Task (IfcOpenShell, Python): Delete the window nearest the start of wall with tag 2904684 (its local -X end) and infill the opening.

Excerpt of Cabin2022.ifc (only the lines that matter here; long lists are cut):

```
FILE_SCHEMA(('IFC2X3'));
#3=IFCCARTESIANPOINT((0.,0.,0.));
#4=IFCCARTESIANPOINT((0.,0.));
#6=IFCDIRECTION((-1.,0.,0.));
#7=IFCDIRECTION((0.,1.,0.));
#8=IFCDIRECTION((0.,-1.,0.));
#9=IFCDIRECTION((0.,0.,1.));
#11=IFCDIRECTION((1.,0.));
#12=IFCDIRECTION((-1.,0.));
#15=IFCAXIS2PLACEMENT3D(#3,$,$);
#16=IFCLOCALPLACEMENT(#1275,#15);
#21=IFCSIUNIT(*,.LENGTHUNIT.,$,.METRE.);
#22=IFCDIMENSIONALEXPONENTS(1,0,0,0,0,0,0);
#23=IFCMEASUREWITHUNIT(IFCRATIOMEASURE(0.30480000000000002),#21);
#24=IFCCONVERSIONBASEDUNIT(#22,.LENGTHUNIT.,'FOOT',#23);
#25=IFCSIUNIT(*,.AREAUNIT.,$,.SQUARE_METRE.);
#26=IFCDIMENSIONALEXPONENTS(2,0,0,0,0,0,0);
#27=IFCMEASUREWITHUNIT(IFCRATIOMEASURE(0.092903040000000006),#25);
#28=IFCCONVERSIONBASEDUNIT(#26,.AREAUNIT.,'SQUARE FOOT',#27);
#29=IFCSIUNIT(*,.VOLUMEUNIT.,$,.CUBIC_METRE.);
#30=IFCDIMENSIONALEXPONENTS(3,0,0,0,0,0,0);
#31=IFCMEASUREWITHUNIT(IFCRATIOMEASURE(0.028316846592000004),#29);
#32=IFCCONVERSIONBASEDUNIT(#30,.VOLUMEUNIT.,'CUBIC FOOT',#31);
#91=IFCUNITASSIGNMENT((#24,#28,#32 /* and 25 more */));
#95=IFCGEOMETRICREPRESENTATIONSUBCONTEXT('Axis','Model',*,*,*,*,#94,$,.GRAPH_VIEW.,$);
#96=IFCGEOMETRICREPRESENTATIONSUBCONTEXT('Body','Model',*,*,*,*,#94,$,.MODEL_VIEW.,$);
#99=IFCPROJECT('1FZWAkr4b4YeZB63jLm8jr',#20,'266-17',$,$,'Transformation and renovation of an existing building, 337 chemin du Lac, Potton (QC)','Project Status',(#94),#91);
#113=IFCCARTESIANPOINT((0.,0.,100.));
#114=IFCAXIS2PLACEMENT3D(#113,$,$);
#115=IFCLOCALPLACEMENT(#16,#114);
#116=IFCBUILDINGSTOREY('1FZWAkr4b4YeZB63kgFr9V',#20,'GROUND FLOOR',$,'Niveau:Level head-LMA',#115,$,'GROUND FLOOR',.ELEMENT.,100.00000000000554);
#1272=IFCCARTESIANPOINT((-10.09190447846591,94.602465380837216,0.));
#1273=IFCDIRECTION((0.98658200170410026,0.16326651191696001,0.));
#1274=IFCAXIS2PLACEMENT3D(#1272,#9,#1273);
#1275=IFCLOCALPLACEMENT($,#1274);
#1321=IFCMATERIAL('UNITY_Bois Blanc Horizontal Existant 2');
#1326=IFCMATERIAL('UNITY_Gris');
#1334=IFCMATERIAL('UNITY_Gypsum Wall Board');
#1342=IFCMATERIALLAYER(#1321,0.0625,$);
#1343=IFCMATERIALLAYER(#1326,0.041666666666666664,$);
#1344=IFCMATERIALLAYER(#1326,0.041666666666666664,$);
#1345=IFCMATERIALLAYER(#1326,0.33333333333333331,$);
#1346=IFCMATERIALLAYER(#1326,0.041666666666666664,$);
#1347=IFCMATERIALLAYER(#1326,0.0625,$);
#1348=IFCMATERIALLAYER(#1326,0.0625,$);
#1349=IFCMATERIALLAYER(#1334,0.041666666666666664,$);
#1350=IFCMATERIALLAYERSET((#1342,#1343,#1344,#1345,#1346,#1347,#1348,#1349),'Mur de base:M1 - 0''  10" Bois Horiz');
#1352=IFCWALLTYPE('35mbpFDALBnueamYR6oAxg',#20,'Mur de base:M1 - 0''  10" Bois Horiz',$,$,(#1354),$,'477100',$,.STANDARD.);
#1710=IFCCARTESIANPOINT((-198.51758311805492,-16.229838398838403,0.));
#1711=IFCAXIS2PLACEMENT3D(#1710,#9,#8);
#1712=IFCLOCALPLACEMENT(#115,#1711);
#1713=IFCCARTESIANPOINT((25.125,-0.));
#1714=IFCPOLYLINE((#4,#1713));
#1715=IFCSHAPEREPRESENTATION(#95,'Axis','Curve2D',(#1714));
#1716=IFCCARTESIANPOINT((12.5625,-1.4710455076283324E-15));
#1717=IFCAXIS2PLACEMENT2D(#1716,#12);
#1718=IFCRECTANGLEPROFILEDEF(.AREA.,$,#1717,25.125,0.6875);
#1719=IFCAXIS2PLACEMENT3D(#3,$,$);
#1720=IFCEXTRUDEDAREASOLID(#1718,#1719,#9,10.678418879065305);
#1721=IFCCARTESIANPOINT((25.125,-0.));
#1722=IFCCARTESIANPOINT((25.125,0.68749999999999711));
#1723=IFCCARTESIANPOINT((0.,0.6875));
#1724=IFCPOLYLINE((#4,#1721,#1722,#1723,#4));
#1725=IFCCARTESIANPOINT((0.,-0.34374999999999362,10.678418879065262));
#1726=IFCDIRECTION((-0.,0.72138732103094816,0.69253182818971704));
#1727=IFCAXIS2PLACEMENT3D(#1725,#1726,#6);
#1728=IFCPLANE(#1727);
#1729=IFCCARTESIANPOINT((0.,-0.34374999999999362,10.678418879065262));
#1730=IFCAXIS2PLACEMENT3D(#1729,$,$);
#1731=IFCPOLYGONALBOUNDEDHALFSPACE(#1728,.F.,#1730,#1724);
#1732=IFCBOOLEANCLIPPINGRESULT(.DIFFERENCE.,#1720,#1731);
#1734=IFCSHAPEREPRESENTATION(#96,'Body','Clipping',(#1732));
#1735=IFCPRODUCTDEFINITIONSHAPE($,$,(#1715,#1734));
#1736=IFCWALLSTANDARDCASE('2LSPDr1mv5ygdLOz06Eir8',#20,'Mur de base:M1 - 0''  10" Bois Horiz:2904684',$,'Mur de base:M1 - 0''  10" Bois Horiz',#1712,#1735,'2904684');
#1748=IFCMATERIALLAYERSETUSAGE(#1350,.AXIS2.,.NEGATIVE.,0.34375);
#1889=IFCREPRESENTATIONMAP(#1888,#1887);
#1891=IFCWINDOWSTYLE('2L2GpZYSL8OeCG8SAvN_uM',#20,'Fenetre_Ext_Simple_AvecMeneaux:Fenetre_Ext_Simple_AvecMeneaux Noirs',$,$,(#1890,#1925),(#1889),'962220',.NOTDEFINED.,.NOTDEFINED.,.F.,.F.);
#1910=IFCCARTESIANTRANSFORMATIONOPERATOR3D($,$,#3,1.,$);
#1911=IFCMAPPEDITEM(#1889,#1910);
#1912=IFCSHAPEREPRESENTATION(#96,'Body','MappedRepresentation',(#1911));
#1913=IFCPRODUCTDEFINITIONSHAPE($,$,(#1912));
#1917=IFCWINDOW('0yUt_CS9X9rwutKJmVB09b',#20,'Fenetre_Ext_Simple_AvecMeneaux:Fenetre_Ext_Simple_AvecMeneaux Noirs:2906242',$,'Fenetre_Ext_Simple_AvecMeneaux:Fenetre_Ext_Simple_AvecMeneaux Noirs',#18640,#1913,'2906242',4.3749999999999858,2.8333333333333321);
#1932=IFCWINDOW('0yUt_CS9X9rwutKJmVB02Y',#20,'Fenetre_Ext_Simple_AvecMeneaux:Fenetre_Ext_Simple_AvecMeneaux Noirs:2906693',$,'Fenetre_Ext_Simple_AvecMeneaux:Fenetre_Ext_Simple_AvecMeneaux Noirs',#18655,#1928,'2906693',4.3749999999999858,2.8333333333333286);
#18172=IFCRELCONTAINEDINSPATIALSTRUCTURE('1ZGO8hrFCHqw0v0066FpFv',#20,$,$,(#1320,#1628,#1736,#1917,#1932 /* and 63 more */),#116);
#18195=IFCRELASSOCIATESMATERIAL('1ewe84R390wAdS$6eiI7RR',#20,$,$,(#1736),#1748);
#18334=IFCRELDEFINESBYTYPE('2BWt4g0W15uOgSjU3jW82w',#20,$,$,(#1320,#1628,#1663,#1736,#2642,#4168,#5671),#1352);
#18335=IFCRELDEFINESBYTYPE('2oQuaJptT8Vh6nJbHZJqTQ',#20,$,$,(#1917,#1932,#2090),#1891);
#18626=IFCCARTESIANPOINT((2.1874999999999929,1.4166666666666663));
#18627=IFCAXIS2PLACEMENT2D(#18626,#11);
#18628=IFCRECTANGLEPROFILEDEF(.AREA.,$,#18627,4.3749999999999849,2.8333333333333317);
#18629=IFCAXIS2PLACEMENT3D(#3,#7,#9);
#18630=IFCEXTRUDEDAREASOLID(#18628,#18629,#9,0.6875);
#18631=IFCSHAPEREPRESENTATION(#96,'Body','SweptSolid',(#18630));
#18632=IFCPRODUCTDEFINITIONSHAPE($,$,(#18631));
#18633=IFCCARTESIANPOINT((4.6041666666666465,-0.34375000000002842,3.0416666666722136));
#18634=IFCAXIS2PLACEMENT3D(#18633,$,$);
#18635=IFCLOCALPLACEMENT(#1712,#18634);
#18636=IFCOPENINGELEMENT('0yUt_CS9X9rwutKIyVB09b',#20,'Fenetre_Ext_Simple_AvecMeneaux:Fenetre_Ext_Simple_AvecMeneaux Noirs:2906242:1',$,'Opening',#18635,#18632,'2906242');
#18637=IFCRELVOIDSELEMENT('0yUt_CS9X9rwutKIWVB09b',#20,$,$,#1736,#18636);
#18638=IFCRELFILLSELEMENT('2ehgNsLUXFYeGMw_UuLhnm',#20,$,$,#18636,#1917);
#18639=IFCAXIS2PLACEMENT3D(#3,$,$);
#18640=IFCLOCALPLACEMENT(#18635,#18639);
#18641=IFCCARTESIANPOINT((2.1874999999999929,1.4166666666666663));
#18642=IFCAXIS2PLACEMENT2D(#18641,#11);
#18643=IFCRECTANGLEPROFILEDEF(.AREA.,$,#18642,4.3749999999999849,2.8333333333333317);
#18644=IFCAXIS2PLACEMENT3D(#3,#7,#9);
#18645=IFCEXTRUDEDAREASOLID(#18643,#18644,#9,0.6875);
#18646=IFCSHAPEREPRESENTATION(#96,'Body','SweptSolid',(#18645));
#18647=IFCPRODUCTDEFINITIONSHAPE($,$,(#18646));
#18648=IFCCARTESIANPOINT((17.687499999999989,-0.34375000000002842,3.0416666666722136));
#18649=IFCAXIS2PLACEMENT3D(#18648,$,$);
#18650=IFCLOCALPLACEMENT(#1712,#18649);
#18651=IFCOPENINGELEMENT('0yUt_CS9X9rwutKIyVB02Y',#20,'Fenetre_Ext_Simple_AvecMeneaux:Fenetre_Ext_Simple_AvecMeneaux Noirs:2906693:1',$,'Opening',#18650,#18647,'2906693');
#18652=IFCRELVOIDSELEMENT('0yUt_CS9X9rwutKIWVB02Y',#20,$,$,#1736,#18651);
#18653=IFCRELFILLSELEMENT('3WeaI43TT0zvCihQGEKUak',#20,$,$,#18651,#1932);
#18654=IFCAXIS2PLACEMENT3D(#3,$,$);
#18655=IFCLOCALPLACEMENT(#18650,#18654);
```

```python
import ifcopenshell
import ifcopenshell.api.feature
import ifcopenshell.api.root
import ifcopenshell.geom
import ifcopenshell.util.shape

model = ifcopenshell.open("Cabin2022.ifc")
settings = ifcopenshell.geom.settings()


def volume(element):
    """Net volume in cubic metres, openings subtracted."""
    shape = ifcopenshell.geom.create_shape(settings, element)
    return ifcopenshell.util.shape.get_volume(shape.geometry)


window = model.by_guid("0yUt_CS9X9rwutKJmVB09b")
opening = window.FillsVoids[0].RelatingOpeningElement
wall = opening.VoidsElements[0].RelatingBuildingElement
before = volume(wall)

ifcopenshell.api.root.remove_product(model, product=window)
ifcopenshell.api.feature.remove_feature(model, feature=opening)

after = volume(wall)

print(f"wall volume {before:.3f} -> {after:.3f} m3")

model.write("Cabin2022_v2.ifc")
```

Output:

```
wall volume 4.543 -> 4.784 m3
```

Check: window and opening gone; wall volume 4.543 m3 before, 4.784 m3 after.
